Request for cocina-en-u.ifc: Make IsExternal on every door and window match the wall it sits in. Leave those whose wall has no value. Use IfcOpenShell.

First a look at what the model holds.

```python
import ifcopenshell
import ifcopenshell.util.element

model = ifcopenshell.open("cocina-en-u.ifc")
print(model.schema)
seen = {}
for e in model.by_type("IfcDoor") + model.by_type("IfcWindow"):
    if not e.FillsVoids:
        continue
    host = e.FillsVoids[0].RelatingOpeningElement.VoidsElements[0].RelatingBuildingElement
    own = ifcopenshell.util.element.get_pset(e, f"Pset_{e.is_a()[3:].removesuffix('StandardCase')}Common", "IsExternal")
    wall = ifcopenshell.util.element.get_pset(host, "Pset_WallCommon", "IsExternal")
    seen[e.is_a(), own, wall] = seen.get((e.is_a(), own, wall), 0) + 1
for (cls, own, wall), count in sorted(seen.items(), key=str):
    print(count, cls, "IsExternal:", own, "| host wall:", wall)
```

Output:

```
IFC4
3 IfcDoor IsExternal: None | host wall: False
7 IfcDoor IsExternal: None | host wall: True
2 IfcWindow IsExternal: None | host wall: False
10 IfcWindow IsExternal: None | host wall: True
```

```python
import ifcopenshell
import ifcopenshell.api.pset
import ifcopenshell.util.element

model = ifcopenshell.open("cocina-en-u.ifc")

count = 0
for ifc_class, pset_name in (("IfcDoor", "Pset_DoorCommon"), ("IfcWindow", "Pset_WindowCommon")):
    for e in model.by_type(ifc_class):
        if not e.FillsVoids:
            continue
        host = e.FillsVoids[0].RelatingOpeningElement.VoidsElements[0].RelatingBuildingElement
        external = ifcopenshell.util.element.get_pset(host, "Pset_WallCommon", "IsExternal")
        if external is None or ifcopenshell.util.element.get_pset(e, pset_name, "IsExternal") == external:
            continue
        pset = ifcopenshell.api.pset.add_pset(model, product=e, name=pset_name)
        ifcopenshell.api.pset.edit_pset(model, pset=pset, properties={"IsExternal": external})
        count += 1

print(count, "updated")

model.write("cocina-en-u_updated.ifc")
```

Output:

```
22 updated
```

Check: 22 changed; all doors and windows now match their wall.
